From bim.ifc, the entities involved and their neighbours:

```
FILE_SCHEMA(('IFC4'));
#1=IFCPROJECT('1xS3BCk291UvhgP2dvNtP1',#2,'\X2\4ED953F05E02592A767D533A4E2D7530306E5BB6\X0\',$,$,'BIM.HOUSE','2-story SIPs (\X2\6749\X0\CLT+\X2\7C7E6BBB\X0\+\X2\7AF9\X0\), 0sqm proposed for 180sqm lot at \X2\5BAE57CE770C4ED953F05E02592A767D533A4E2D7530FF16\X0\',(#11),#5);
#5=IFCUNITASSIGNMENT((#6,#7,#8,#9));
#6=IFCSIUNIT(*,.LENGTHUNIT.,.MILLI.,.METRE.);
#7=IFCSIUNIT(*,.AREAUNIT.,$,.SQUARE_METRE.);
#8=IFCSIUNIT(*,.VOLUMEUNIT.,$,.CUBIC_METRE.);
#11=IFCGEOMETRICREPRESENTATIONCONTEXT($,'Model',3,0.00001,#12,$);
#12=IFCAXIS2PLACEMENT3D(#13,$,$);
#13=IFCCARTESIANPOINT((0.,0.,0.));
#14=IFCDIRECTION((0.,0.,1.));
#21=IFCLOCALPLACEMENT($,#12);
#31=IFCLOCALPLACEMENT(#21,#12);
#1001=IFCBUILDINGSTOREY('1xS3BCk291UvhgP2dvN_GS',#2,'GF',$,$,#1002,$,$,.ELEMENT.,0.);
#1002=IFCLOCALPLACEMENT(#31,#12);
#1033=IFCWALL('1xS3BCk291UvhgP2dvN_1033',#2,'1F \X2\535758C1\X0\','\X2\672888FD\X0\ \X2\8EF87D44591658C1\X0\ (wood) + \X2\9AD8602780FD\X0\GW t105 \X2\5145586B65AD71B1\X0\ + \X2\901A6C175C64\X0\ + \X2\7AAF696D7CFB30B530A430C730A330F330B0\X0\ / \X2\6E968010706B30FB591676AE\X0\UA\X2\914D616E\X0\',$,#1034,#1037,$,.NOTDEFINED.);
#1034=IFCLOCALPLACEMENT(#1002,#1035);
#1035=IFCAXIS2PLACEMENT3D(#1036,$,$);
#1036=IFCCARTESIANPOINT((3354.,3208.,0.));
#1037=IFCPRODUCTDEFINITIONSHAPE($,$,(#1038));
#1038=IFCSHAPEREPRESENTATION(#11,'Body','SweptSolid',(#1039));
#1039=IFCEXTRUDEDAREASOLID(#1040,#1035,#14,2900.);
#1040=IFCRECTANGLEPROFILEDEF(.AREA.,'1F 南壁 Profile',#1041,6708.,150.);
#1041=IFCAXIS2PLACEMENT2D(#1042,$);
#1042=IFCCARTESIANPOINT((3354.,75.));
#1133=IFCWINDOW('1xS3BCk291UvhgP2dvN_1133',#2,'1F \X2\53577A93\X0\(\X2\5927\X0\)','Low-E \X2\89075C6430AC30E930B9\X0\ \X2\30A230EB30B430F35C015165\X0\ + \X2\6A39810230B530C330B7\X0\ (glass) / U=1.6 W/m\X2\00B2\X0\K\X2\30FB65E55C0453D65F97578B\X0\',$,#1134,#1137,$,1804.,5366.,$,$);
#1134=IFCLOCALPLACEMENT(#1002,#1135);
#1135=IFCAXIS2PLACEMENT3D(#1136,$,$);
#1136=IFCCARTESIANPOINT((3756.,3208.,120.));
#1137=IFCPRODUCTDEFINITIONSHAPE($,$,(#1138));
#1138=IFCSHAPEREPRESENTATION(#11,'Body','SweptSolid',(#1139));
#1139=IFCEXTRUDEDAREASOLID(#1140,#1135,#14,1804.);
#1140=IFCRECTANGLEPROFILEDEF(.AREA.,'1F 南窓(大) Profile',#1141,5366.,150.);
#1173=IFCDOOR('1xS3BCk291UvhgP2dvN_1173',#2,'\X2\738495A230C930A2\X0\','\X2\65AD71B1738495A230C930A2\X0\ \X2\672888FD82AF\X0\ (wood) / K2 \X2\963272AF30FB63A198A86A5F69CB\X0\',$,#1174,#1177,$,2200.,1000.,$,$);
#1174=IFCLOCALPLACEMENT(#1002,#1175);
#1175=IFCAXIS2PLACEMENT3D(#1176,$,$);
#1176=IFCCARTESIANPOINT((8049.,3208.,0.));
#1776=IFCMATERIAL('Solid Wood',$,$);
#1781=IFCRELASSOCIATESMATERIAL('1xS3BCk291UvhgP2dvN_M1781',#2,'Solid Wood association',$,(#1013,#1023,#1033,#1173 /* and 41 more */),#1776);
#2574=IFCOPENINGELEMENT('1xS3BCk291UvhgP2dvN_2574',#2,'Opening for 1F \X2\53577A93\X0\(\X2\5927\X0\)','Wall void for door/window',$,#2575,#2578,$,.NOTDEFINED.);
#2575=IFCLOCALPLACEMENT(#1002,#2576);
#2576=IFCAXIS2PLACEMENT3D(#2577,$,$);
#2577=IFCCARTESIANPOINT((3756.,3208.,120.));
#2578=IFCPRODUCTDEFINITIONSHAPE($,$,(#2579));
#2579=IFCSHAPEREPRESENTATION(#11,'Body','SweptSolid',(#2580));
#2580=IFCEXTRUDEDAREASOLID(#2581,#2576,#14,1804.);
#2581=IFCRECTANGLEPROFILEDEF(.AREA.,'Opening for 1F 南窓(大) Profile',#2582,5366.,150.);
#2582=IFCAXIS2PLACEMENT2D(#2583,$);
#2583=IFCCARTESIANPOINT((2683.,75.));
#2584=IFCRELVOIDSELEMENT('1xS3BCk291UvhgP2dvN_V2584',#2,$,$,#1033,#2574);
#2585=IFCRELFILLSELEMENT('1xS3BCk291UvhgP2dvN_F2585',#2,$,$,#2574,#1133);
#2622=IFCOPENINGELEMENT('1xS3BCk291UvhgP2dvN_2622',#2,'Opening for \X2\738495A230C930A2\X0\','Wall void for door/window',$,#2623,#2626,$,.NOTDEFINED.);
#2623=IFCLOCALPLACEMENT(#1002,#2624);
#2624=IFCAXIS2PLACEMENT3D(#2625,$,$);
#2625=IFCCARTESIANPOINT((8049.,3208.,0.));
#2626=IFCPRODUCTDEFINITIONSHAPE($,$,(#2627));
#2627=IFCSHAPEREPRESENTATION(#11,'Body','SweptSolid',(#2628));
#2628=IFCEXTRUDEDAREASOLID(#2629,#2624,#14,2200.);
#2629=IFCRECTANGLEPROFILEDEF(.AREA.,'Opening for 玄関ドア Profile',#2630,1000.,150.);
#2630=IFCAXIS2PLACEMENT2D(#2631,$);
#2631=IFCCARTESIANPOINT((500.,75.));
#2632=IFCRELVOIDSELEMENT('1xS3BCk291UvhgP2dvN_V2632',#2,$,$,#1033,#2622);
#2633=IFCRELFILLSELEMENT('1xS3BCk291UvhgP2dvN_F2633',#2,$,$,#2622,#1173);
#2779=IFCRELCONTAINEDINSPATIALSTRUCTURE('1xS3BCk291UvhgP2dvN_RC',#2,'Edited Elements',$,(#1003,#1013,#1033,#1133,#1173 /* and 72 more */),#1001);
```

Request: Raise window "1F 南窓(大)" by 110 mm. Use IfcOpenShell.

```python
import numpy as np
import ifcopenshell
import ifcopenshell.api.geometry
import ifcopenshell.util.placement
import ifcopenshell.util.unit

model = ifcopenshell.open("bim.ifc")
unit_scale = ifcopenshell.util.unit.calculate_unit_scale(model)

window = model.by_guid("1xS3BCk291UvhgP2dvN_1133")
opening = window.FillsVoids[0].RelatingOpeningElement
dz = 110.0

shift = np.array([0.0, 0.0, dz])
# The window is not placed relative to its opening, so move both.
for product in (opening, window):
    matrix = ifcopenshell.util.placement.get_local_placement(product.ObjectPlacement)
    matrix[:3, 3] += shift
    ifcopenshell.api.geometry.edit_object_placement(model, product=product, matrix=matrix, is_si=False)

print(f"moved by {dz * unit_scale:+.3f} m")

model.write("bim_edited.ifc")
```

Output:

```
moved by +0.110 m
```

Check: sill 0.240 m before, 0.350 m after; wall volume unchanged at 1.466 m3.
